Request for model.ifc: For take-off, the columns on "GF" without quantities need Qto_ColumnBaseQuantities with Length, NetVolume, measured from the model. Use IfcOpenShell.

First a look at what the model holds.

```python
import ifcopenshell
import ifcopenshell.util.element
import ifcopenshell.util.unit

model = ifcopenshell.open("model.ifc")
print(model.schema)
for unit_type in ("LENGTHUNIT", "AREAUNIT", "VOLUMEUNIT"):
    print(unit_type, ifcopenshell.util.unit.calculate_unit_scale(model, unit_type))
storey = next(s for s in model.by_type("IfcBuildingStorey") if s.Name == "GF")
columns = [e for e in ifcopenshell.util.element.get_decomposition(storey) if e.is_a("IfcColumn")]
for e in sorted(columns, key=lambda e: e.id()):
    print(e.id(), e.is_a(), e.Name, list(ifcopenshell.util.element.get_psets(e, qtos_only=True)), sep=" | ")
```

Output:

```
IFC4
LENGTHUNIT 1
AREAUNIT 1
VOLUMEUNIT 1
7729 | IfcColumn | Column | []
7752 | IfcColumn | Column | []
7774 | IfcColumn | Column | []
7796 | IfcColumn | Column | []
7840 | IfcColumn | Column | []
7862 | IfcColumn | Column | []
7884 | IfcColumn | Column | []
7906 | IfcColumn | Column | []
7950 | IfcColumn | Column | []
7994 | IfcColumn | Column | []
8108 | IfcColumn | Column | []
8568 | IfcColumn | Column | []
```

```python
import ifcopenshell
import ifcopenshell.api.pset
import ifcopenshell.geom
import ifcopenshell.util.element
import ifcopenshell.util.shape
import ifcopenshell.util.unit

model = ifcopenshell.open("model.ifc")
unit_scale = ifcopenshell.util.unit.calculate_unit_scale(model)
volume_scale = ifcopenshell.util.unit.calculate_unit_scale(model, "VOLUMEUNIT")
settings = ifcopenshell.geom.settings()

storey = next(s for s in model.by_type("IfcBuildingStorey") if s.Name == "GF")
columns = [e for e in ifcopenshell.util.element.get_decomposition(storey) if e.is_a("IfcColumn")]

for e in sorted(columns, key=lambda e: e.id()):
    if ifcopenshell.util.element.get_psets(e, qtos_only=True, should_inherit=False):
        continue
    # Geometry comes back in metres, in the element's own axes.
    shape = ifcopenshell.geom.create_shape(settings, e)
    values = {
        "Length": ifcopenshell.util.shape.get_z(shape.geometry) / unit_scale,
        "NetVolume": ifcopenshell.util.shape.get_volume(shape.geometry) / volume_scale,
    }
    qto = ifcopenshell.api.pset.add_qto(model, product=e, name="Qto_ColumnBaseQuantities")
    ifcopenshell.api.pset.edit_qto(model, qto=qto, properties=values)
    print(e.id(), {k: round(v, 3) for k, v in values.items()})

model.write("model_rev.ifc")
```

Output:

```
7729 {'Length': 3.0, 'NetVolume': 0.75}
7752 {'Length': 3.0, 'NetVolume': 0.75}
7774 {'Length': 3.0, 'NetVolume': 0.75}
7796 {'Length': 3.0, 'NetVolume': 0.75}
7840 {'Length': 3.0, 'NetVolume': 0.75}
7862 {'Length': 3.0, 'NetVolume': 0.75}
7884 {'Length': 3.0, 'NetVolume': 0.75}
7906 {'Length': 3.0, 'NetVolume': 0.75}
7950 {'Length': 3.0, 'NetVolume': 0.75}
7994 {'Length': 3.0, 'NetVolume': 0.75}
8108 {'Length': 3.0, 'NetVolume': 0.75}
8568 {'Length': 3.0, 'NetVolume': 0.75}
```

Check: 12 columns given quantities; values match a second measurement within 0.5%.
